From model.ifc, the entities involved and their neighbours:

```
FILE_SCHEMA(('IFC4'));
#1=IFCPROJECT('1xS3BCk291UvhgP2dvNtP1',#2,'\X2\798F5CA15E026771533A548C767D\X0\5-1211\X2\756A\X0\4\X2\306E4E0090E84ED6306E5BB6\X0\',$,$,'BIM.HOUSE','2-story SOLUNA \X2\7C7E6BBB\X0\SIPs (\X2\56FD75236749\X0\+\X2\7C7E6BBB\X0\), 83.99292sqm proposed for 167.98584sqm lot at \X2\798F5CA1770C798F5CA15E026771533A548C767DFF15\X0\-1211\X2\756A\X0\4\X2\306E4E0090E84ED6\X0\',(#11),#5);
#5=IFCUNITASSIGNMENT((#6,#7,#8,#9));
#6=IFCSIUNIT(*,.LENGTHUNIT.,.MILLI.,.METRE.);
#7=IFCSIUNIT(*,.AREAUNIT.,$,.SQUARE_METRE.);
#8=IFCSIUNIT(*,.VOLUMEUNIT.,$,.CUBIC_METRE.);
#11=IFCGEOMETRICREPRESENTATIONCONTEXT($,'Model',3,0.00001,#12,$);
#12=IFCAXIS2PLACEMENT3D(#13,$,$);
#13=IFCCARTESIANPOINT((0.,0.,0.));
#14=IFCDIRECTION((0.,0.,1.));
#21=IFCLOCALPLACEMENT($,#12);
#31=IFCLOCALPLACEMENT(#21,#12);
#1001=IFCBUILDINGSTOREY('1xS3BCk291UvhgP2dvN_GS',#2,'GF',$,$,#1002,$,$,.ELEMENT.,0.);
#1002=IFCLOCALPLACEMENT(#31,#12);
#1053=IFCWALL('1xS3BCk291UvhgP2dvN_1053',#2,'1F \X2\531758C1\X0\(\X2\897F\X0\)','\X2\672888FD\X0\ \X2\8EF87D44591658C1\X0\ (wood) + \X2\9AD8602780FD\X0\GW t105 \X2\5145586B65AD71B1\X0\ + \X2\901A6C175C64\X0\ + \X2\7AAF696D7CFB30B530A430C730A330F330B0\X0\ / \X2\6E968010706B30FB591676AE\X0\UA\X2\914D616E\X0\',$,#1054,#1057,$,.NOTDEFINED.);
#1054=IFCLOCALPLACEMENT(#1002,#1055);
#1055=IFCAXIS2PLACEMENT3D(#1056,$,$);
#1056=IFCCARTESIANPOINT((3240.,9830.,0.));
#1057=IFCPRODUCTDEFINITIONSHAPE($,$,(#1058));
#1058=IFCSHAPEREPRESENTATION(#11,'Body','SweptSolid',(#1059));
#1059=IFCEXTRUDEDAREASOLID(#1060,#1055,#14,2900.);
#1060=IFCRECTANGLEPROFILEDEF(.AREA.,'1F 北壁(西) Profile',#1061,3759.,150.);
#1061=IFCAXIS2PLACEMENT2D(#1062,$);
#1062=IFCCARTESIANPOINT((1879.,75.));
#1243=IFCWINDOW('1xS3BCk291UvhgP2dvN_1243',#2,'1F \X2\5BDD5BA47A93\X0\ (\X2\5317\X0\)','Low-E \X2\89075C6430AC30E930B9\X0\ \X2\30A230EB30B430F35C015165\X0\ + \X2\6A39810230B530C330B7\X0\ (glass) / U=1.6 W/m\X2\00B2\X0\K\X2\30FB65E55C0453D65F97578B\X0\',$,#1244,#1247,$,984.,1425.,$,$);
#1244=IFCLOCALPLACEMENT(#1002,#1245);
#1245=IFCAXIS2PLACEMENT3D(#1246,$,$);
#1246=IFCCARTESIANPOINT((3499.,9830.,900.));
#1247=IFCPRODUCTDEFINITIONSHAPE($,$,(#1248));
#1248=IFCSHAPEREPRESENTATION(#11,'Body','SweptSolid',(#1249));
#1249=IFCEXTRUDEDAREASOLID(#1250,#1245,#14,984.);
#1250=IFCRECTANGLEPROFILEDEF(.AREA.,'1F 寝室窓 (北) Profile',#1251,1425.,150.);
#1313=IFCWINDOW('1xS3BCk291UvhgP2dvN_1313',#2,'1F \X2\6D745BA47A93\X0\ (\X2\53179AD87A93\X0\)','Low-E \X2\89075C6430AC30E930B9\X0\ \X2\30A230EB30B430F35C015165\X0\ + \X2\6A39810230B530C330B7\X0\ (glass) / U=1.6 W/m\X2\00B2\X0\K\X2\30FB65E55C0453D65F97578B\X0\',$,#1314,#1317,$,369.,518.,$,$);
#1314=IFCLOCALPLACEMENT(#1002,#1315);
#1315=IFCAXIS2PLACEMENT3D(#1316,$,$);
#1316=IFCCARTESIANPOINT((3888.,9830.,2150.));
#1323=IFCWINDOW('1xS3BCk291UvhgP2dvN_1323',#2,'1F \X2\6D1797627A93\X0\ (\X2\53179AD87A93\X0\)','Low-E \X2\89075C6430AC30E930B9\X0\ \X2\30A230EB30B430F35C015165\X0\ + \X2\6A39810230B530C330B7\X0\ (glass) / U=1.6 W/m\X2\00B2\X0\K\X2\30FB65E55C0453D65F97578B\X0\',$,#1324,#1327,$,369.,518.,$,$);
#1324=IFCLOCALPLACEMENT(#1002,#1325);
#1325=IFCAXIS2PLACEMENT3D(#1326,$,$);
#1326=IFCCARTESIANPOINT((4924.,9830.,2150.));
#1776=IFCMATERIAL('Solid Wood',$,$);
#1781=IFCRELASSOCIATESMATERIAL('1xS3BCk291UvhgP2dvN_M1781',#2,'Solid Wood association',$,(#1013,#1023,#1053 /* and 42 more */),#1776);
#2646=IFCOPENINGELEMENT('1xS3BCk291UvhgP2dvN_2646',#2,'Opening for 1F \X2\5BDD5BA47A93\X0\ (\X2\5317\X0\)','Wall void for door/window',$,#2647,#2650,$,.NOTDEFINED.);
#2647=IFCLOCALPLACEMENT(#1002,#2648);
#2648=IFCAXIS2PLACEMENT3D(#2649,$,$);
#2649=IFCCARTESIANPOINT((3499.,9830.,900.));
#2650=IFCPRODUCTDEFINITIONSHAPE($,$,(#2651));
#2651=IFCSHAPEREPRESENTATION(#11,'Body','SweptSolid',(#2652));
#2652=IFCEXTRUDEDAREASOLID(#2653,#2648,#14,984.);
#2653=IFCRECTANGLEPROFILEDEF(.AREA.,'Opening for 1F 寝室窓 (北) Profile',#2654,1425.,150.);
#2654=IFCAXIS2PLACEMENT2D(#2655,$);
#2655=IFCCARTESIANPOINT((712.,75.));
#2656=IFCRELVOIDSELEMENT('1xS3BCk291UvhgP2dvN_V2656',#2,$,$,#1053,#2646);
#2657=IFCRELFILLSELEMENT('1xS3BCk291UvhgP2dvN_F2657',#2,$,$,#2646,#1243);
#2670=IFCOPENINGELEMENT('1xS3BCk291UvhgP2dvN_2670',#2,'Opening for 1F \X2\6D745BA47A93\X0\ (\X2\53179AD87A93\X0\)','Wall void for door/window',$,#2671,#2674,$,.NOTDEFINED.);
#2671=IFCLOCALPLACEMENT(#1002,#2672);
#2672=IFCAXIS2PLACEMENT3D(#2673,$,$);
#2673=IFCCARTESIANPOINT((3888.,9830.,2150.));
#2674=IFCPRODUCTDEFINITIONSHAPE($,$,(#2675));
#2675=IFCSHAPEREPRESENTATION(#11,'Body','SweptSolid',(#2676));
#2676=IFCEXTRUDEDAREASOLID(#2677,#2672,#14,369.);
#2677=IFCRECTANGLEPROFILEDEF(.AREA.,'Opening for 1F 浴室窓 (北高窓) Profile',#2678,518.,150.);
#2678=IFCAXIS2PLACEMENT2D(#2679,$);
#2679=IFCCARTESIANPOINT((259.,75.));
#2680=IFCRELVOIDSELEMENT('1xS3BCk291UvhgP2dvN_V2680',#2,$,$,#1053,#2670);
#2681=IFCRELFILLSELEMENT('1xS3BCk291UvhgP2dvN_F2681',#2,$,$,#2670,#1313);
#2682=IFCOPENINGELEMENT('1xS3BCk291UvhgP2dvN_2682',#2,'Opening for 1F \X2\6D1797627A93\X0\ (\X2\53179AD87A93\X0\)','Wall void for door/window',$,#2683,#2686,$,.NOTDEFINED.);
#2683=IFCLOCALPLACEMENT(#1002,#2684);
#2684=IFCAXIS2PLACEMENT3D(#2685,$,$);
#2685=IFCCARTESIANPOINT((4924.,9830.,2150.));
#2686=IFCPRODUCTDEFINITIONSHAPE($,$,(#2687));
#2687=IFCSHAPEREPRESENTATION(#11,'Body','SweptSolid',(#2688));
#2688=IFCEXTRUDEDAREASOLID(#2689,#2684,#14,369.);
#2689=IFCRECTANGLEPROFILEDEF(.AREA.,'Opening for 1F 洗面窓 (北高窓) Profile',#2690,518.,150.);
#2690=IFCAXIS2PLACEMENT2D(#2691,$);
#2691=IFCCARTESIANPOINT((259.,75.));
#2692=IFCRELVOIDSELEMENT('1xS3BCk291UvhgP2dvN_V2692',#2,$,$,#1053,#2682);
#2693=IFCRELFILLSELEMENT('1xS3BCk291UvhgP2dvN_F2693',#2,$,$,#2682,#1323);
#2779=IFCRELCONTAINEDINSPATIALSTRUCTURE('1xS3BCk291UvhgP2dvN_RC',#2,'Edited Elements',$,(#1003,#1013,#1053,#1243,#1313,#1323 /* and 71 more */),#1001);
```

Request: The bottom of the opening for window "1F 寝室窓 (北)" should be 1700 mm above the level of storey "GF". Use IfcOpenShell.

```python
import numpy as np
import ifcopenshell
import ifcopenshell.api.geometry
import ifcopenshell.geom
import ifcopenshell.util.element
import ifcopenshell.util.placement
import ifcopenshell.util.shape
import ifcopenshell.util.unit

model = ifcopenshell.open("model.ifc")
unit_scale = ifcopenshell.util.unit.calculate_unit_scale(model)

window = model.by_guid("1xS3BCk291UvhgP2dvN_1243")
opening = window.FillsVoids[0].RelatingOpeningElement
storey = ifcopenshell.util.element.get_container(window, ifc_class="IfcBuildingStorey")
level = ifcopenshell.util.placement.get_local_placement(storey.ObjectPlacement)[2, 3]

# The opening's origin need not be at the sill, so measure its lowest point.
shape = ifcopenshell.geom.create_shape(ifcopenshell.geom.settings(), opening)
bottom = ifcopenshell.util.shape.get_shape_bottom_elevation(shape, shape.geometry) / unit_scale
dz = level + 1700.0 - bottom

shift = np.array([0.0, 0.0, dz])
# The window is not placed relative to its opening, so move both.
for product in (opening, window):
    matrix = ifcopenshell.util.placement.get_local_placement(product.ObjectPlacement)
    matrix[:3, 3] += shift
    ifcopenshell.api.geometry.edit_object_placement(model, product=product, matrix=matrix, is_si=False)

print(f"moved by {dz * unit_scale:+.3f} m")

model.write("model_rev.ifc")
```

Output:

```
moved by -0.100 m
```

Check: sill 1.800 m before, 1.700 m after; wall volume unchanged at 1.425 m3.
